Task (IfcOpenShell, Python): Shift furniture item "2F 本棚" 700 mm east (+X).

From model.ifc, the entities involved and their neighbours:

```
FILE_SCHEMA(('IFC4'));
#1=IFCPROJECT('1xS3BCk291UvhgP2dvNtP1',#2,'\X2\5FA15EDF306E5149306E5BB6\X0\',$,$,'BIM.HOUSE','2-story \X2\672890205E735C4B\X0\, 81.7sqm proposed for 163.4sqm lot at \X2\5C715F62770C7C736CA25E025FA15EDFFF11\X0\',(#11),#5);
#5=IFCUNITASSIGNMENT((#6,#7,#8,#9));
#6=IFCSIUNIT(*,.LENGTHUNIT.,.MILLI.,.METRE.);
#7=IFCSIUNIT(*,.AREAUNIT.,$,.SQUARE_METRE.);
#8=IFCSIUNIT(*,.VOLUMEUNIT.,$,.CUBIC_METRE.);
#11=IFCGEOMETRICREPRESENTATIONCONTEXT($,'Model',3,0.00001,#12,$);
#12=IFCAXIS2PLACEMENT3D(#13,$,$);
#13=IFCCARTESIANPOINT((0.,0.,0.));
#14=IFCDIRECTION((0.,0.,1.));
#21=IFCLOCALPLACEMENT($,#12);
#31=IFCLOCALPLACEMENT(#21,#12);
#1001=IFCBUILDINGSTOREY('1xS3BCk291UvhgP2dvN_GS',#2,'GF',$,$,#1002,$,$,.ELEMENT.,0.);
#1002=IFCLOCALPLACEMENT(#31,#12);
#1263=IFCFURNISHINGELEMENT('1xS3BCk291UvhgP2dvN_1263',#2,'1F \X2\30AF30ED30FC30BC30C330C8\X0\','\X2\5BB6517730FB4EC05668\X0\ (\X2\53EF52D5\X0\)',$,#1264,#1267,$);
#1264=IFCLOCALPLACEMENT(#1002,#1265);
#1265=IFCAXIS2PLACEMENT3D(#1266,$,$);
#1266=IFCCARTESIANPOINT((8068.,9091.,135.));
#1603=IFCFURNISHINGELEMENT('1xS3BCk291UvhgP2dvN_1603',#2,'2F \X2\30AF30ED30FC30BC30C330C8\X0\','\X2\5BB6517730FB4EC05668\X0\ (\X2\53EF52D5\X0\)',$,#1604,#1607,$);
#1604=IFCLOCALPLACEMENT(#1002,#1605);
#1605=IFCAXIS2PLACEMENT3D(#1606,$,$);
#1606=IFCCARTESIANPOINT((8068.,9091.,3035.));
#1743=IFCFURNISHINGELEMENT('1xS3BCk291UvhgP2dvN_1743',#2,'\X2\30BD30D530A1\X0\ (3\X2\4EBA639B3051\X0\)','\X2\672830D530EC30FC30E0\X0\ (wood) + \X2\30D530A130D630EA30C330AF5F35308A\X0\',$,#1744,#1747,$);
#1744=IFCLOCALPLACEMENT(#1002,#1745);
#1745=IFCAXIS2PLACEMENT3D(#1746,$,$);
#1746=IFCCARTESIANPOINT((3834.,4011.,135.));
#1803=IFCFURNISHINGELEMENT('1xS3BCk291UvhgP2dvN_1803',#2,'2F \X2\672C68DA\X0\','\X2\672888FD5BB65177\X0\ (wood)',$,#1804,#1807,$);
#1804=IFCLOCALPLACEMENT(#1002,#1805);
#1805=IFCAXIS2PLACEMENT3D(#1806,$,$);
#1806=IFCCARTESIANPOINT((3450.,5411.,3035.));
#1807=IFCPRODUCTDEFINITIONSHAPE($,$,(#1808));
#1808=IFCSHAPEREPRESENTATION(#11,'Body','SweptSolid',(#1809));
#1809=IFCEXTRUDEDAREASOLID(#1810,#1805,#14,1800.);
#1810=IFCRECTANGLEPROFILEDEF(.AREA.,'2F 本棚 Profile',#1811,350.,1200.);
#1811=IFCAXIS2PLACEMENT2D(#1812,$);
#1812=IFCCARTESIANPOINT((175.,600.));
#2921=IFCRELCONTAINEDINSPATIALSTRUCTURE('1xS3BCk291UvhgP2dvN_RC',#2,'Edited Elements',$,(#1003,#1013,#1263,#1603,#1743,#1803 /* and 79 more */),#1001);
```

```python
import ifcopenshell
import ifcopenshell.api.geometry
import ifcopenshell.util.placement
import ifcopenshell.util.unit

model = ifcopenshell.open("model.ifc")
unit_scale = ifcopenshell.util.unit.calculate_unit_scale(model)

item = model.by_guid("1xS3BCk291UvhgP2dvN_1803")
matrix = ifcopenshell.util.placement.get_local_placement(item.ObjectPlacement)
matrix[0, 3] += 0.7 / unit_scale
ifcopenshell.api.geometry.edit_object_placement(model, product=item, matrix=matrix, is_si=False)

print(ifcopenshell.util.placement.get_local_placement(item.ObjectPlacement).round(3) + 0.0)

model.write("model_v2.ifc")
```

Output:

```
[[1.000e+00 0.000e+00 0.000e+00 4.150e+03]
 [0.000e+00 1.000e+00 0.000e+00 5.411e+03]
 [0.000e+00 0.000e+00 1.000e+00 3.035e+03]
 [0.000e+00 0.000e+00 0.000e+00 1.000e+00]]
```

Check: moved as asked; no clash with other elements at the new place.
